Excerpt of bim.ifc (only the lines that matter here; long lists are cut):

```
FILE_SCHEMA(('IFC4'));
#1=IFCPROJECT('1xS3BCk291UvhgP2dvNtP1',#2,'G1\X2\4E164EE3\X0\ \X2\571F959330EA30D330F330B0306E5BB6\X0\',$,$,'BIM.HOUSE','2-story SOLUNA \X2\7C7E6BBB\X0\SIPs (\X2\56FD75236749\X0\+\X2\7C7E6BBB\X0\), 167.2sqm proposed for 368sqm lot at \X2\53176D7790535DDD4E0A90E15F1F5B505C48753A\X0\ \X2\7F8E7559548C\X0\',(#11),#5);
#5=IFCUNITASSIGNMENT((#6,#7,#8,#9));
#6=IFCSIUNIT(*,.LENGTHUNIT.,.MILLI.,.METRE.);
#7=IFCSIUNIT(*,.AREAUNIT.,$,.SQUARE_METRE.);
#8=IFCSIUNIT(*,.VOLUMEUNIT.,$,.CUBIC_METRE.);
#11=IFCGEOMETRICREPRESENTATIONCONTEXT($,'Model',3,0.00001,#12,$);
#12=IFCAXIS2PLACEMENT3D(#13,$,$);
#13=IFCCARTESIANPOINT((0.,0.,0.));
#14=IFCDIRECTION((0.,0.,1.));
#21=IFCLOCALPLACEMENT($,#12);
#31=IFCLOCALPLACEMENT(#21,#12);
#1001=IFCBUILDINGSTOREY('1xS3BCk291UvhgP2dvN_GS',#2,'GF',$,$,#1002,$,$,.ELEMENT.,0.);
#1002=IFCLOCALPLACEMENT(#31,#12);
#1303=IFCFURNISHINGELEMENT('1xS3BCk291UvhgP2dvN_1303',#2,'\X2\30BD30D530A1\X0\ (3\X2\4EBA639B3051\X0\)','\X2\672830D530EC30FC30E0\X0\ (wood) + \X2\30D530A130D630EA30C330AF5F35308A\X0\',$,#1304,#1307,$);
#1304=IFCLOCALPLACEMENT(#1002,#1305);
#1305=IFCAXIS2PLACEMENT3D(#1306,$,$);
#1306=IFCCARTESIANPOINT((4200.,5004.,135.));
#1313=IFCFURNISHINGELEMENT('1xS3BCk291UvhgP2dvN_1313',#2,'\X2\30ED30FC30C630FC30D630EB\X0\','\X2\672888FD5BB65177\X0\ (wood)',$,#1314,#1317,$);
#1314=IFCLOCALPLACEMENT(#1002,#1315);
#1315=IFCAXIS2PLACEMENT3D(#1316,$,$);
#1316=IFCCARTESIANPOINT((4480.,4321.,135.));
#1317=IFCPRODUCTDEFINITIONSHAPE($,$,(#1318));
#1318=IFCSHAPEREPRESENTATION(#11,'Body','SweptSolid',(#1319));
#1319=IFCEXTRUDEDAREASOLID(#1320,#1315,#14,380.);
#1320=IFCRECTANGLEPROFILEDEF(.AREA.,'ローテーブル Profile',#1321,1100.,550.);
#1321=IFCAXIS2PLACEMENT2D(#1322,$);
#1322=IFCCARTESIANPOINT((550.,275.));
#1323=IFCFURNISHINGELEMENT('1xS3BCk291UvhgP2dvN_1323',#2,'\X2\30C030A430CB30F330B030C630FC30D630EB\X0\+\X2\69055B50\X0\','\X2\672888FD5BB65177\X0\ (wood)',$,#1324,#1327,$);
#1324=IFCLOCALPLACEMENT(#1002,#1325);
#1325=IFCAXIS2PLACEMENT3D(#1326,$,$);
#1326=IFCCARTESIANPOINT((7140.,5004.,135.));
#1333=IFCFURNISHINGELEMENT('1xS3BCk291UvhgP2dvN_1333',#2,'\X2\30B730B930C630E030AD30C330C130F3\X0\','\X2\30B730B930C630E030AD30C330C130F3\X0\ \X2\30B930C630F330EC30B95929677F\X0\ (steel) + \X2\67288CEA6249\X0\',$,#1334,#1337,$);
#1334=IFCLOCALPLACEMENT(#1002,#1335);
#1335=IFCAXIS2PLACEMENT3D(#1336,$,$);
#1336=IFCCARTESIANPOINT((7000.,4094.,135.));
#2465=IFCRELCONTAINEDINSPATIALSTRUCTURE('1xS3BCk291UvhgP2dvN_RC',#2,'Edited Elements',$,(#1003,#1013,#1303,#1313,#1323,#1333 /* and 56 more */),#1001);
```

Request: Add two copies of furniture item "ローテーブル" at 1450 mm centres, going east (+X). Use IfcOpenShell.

```python
import numpy as np
import ifcopenshell
import ifcopenshell.api.geometry
import ifcopenshell.api.root
import ifcopenshell.util.element
import ifcopenshell.util.placement

model = ifcopenshell.open("bim.ifc")


def reuse_history(source, copy):
    """copy_class also copies each property set's owner history, people and application; keep the originals."""
    for rel in copy.IsDefinedBy:
        if rel.is_a("IfcRelDefinesByProperties") and (history := rel.RelatingPropertyDefinition.OwnerHistory):
            rel.RelatingPropertyDefinition.OwnerHistory = source.OwnerHistory
            ifcopenshell.util.element.remove_deep2(model, history)


source = model.by_id(1313)
base = ifcopenshell.util.placement.get_local_placement(source.ObjectPlacement)
step = np.array([1.0, 0.0, 0.0]) * 1450.0

for i in range(1, 3):
    copy = ifcopenshell.api.root.copy_class(model, product=source)
    copy.Representation = ifcopenshell.util.element.copy_deep(
        model, source.Representation, exclude=["IfcGeometricRepresentationContext", "IfcRepresentationMap"]
    )
    reuse_history(source, copy)
    matrix = base.copy()
    matrix[:3, 3] += i * step
    print("added at", matrix[:3, 3].round(3) + 0.0)
    ifcopenshell.api.geometry.edit_object_placement(model, product=copy, matrix=matrix, is_si=False)

model.write("bim_updated.ifc")
```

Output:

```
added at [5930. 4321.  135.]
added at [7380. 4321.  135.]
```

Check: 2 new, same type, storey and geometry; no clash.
